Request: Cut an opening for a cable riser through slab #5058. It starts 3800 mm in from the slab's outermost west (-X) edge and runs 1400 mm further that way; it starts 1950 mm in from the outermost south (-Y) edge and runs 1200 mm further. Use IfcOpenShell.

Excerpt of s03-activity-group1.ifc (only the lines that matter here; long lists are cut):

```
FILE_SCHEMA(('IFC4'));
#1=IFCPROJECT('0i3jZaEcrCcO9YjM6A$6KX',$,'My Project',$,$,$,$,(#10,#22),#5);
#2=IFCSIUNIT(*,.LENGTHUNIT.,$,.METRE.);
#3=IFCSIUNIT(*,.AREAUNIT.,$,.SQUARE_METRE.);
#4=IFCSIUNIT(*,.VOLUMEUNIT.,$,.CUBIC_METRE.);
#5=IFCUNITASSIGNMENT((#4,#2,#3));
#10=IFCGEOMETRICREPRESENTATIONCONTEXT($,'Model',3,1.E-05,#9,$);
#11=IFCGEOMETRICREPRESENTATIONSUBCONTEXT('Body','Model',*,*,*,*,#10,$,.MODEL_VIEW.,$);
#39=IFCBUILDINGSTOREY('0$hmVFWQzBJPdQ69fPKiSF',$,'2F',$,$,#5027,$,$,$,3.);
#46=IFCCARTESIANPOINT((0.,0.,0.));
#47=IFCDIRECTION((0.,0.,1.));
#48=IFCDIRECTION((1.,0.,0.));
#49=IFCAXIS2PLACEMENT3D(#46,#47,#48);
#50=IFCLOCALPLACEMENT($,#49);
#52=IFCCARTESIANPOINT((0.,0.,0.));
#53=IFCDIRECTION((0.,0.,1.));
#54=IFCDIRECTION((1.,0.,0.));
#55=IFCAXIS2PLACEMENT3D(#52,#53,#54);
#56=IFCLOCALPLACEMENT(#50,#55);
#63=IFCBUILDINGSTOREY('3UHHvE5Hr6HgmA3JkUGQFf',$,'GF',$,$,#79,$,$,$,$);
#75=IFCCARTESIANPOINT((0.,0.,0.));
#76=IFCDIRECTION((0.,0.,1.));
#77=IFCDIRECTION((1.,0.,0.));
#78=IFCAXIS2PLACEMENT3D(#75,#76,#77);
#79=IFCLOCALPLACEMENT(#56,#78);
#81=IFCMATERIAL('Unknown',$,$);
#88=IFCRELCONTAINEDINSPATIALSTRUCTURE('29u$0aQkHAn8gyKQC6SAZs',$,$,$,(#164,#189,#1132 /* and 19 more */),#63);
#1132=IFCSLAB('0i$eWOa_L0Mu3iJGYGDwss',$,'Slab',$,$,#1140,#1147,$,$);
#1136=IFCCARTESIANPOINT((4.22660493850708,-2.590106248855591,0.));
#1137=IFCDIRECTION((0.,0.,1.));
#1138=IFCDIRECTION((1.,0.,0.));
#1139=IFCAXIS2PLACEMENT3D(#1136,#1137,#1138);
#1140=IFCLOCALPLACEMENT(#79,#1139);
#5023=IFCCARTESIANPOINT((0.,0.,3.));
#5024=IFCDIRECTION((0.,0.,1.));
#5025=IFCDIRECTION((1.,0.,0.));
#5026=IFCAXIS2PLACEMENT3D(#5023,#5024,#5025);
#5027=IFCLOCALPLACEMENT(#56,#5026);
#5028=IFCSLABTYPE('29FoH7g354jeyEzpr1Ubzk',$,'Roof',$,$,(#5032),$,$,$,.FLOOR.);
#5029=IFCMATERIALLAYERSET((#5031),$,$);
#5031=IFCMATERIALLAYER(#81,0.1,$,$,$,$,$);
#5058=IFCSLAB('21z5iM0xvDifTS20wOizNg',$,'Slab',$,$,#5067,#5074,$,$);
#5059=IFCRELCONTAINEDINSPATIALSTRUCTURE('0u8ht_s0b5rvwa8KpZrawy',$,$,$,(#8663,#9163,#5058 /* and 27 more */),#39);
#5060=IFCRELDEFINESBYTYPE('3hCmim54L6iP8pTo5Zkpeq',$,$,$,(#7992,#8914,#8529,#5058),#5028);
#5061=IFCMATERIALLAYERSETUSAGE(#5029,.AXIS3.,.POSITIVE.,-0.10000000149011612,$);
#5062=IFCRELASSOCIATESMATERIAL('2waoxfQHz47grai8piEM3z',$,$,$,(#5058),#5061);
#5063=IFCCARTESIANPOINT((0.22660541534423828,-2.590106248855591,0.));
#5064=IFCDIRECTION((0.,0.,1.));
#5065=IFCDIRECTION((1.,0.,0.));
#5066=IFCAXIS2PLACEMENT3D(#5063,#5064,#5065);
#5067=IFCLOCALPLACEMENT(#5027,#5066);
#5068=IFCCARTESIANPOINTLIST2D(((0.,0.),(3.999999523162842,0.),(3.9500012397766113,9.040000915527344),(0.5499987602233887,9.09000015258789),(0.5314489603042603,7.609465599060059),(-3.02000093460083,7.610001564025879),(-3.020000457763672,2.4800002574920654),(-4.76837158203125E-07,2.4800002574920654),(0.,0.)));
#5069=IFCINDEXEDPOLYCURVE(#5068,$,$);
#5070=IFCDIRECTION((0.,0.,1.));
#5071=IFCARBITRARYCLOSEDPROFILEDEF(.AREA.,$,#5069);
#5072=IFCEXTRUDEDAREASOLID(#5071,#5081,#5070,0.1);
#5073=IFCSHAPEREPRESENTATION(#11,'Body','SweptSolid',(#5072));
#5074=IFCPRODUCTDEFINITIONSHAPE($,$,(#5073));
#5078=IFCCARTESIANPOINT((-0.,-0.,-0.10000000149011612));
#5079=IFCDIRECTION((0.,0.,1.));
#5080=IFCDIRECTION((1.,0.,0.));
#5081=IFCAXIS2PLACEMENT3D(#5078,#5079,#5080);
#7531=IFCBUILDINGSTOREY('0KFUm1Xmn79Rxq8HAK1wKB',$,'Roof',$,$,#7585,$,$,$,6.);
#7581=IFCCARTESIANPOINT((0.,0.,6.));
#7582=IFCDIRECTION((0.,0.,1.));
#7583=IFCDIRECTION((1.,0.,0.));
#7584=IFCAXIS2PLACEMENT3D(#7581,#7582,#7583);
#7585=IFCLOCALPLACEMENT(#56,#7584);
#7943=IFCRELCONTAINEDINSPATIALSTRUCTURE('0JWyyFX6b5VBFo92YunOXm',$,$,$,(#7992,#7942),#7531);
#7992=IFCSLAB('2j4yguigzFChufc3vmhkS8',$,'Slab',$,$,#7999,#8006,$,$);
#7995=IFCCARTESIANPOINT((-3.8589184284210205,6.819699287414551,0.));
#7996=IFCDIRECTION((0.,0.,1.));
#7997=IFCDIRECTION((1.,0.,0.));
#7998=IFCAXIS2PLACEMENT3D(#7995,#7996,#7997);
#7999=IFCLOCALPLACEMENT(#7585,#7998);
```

```python
import numpy as np
import ifcopenshell
import ifcopenshell.api.feature
import ifcopenshell.api.geometry
import ifcopenshell.api.root
import ifcopenshell.geom
import ifcopenshell.util.placement
import ifcopenshell.util.representation
import ifcopenshell.util.shape
import ifcopenshell.util.unit

model = ifcopenshell.open("s03-activity-group1.ifc")
unit_scale = ifcopenshell.util.unit.calculate_unit_scale(model)
settings = ifcopenshell.geom.settings()


def volume(element):
    """Net volume in cubic metres, openings subtracted."""
    shape = ifcopenshell.geom.create_shape(settings, element)
    return ifcopenshell.util.shape.get_volume(shape.geometry)


slab = model.by_id(5058)
before = volume(slab)

# Extent in the slab's own axes, in metres. The edges named are its -X and -Y sides.
slab_shape = ifcopenshell.geom.create_shape(settings, slab)
vertices = ifcopenshell.util.shape.get_vertices(slab_shape.geometry)
x_min, y_min, bottom = vertices.min(axis=0)
top = vertices[:, 2].max()

opening = ifcopenshell.api.root.create_entity(model, ifc_class="IfcOpeningElement", name="Cable riser opening", predefined_type="OPENING")
context = ifcopenshell.util.representation.get_context(model, "Model", "Body", "MODEL_VIEW")
width, depth = 1.4, 1.2
outline = [(0.0, 0.0), (width, 0.0), (width, depth), (0.0, depth), (0.0, 0.0)]
# Overshoot both faces by 50 mm so the cut is clean.
shape = ifcopenshell.api.geometry.add_slab_representation(
    model, context=context, depth=top - bottom + 0.1, polyline=outline
)
ifcopenshell.api.geometry.assign_representation(model, product=opening, representation=shape)

matrix = ifcopenshell.util.placement.get_local_placement(slab.ObjectPlacement)
matrix[:, 3] = matrix @ np.append(np.array([x_min + 3.8, y_min + 1.95, bottom - 0.05]) / unit_scale, 1.0)
ifcopenshell.api.geometry.edit_object_placement(model, product=opening, matrix=matrix, is_si=False)
ifcopenshell.api.feature.add_feature(model, feature=opening, element=slab)

after = volume(slab)

print(f"slab volume {before:.3f} -> {after:.3f} m3")

model.write("s03-activity-group1-out.ifc")
```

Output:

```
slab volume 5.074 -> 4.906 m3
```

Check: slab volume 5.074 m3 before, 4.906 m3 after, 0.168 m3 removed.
